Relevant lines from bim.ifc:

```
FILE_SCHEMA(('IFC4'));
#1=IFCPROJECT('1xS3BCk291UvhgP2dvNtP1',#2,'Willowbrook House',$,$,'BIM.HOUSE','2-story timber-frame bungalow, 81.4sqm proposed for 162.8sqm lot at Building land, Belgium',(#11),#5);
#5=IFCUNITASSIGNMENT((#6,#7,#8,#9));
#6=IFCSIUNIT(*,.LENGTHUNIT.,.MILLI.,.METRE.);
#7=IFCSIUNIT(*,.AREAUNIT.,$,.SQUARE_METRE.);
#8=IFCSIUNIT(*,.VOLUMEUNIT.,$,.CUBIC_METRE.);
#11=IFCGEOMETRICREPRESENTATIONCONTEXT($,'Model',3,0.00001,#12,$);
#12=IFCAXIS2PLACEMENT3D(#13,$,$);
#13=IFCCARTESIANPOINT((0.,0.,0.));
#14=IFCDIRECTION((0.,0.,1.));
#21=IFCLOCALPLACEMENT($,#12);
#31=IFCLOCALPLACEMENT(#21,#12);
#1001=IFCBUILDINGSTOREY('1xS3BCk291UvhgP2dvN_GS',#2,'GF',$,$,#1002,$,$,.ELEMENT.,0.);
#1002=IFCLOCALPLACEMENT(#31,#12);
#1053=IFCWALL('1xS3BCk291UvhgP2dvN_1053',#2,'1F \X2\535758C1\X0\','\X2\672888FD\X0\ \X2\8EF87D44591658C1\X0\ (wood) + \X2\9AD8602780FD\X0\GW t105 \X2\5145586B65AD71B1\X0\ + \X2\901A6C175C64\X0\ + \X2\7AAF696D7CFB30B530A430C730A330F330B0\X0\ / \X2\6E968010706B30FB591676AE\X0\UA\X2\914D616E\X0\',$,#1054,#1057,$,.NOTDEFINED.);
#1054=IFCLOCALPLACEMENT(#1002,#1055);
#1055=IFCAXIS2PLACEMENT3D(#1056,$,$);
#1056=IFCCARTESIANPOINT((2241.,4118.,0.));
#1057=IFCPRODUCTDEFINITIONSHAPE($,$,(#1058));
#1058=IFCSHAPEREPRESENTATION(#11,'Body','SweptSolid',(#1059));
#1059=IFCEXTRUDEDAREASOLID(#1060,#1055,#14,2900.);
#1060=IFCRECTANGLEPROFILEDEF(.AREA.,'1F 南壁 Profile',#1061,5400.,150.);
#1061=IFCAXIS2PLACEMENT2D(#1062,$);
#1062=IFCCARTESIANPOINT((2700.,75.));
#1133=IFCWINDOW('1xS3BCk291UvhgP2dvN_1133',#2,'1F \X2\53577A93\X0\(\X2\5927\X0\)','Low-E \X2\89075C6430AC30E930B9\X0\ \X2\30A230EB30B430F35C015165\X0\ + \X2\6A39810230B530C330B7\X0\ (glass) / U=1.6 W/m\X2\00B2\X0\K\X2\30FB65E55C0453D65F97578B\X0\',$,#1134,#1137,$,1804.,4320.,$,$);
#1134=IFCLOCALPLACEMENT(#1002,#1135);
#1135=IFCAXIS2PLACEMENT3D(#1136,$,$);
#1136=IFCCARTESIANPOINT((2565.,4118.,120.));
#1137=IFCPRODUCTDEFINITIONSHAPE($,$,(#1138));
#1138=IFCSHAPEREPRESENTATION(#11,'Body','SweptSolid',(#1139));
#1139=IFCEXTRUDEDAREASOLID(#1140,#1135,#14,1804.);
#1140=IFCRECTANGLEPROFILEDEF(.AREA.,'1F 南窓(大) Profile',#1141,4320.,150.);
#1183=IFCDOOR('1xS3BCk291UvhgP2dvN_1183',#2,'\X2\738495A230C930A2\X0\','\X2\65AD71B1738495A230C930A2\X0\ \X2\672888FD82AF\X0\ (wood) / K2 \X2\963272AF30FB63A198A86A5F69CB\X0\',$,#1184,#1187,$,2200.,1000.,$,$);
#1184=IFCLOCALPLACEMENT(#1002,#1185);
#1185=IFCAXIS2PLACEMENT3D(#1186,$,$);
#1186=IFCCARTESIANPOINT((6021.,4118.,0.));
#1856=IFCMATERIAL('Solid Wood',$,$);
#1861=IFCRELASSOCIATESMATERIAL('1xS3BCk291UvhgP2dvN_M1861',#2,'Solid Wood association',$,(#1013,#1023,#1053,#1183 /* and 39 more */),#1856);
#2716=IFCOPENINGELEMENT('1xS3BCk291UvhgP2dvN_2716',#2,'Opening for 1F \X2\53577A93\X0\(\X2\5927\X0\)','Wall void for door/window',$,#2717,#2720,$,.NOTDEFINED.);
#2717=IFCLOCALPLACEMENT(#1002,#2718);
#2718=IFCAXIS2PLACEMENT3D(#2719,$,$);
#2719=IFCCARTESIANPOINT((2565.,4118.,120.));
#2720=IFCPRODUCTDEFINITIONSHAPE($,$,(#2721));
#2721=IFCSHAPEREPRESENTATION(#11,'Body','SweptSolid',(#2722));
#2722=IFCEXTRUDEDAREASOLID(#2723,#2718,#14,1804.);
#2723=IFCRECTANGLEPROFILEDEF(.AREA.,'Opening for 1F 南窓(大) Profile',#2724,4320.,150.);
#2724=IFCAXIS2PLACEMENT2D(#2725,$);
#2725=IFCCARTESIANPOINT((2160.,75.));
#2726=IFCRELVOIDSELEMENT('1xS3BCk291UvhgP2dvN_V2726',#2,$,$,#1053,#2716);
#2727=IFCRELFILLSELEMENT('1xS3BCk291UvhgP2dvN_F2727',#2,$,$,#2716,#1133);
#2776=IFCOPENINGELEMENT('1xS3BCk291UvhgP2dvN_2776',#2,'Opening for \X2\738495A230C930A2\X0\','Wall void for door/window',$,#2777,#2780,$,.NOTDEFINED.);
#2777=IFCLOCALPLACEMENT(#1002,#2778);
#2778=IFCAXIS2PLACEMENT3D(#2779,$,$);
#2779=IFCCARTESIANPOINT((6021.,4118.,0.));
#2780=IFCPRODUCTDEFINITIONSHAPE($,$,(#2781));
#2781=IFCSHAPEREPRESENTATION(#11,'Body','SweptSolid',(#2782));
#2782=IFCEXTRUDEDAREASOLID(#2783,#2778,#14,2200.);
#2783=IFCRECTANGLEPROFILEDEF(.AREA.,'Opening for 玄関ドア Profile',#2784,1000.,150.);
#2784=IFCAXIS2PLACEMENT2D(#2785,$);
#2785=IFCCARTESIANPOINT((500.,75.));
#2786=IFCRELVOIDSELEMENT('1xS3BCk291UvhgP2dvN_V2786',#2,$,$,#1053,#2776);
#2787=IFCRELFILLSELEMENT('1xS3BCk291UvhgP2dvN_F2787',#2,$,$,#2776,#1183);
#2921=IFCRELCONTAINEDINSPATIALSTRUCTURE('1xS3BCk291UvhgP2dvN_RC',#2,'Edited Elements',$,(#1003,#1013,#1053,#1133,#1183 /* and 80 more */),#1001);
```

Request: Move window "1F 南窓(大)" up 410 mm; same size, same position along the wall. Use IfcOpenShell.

```python
import numpy as np
import ifcopenshell
import ifcopenshell.api.geometry
import ifcopenshell.util.placement
import ifcopenshell.util.unit

model = ifcopenshell.open("bim.ifc")
unit_scale = ifcopenshell.util.unit.calculate_unit_scale(model)

window = model.by_id(1133)
opening = window.FillsVoids[0].RelatingOpeningElement
dz = 410.0

shift = np.array([0.0, 0.0, dz])
# The window is not placed relative to its opening, so move both.
for product in (opening, window):
    matrix = ifcopenshell.util.placement.get_local_placement(product.ObjectPlacement)
    matrix[:3, 3] += shift
    ifcopenshell.api.geometry.edit_object_placement(model, product=product, matrix=matrix, is_si=False)

print(f"moved by {dz * unit_scale:+.3f} m")

model.write("bim_edited.ifc")
```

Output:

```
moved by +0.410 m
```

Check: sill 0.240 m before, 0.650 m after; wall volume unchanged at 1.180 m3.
